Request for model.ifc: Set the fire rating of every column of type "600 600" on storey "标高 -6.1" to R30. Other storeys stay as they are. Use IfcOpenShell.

First a look at what the model holds.

```python
import ifcopenshell
import ifcopenshell.util.element

model = ifcopenshell.open("model.ifc")
print(model.schema)
storey = next(s for s in model.by_type("IfcBuildingStorey") if s.Name == "标高 -6.1")
columns = [e for e in ifcopenshell.util.element.get_decomposition(storey) if e.is_a("IfcColumn")]
seen = {}
for e in columns:
    element_type = ifcopenshell.util.element.get_type(e)
    key = (element_type.Name if element_type != e and element_type else None, ifcopenshell.util.element.get_pset(e, "Pset_ColumnCommon", "FireRating"))
    seen[key] = seen.get(key, 0) + 1
for (name, value), count in sorted(seen.items(), key=str):
    print(count, "x", name, "|", value)
```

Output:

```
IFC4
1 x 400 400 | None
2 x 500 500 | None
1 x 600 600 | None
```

```python
import ifcopenshell
import ifcopenshell.api.pset
import ifcopenshell.util.element

model = ifcopenshell.open("model.ifc")

storey = next(s for s in model.by_type("IfcBuildingStorey") if s.Name == "标高 -6.1")
columns = [e for e in ifcopenshell.util.element.get_decomposition(storey) if e.is_a("IfcColumn")]

count = 0
for e in columns:
    element_type = ifcopenshell.util.element.get_type(e)
    if element_type in (None, e) or element_type.Name != "600 600":
        continue
    # add_pset returns the element's existing set when there is one.
    pset = ifcopenshell.api.pset.add_pset(model, product=e, name="Pset_ColumnCommon")
    ifcopenshell.api.pset.edit_pset(model, pset=pset, properties={"FireRating": "R30"})
    count += 1

print(count, "columns updated")

model.write("model-out.ifc")
```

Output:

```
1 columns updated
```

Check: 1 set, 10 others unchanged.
